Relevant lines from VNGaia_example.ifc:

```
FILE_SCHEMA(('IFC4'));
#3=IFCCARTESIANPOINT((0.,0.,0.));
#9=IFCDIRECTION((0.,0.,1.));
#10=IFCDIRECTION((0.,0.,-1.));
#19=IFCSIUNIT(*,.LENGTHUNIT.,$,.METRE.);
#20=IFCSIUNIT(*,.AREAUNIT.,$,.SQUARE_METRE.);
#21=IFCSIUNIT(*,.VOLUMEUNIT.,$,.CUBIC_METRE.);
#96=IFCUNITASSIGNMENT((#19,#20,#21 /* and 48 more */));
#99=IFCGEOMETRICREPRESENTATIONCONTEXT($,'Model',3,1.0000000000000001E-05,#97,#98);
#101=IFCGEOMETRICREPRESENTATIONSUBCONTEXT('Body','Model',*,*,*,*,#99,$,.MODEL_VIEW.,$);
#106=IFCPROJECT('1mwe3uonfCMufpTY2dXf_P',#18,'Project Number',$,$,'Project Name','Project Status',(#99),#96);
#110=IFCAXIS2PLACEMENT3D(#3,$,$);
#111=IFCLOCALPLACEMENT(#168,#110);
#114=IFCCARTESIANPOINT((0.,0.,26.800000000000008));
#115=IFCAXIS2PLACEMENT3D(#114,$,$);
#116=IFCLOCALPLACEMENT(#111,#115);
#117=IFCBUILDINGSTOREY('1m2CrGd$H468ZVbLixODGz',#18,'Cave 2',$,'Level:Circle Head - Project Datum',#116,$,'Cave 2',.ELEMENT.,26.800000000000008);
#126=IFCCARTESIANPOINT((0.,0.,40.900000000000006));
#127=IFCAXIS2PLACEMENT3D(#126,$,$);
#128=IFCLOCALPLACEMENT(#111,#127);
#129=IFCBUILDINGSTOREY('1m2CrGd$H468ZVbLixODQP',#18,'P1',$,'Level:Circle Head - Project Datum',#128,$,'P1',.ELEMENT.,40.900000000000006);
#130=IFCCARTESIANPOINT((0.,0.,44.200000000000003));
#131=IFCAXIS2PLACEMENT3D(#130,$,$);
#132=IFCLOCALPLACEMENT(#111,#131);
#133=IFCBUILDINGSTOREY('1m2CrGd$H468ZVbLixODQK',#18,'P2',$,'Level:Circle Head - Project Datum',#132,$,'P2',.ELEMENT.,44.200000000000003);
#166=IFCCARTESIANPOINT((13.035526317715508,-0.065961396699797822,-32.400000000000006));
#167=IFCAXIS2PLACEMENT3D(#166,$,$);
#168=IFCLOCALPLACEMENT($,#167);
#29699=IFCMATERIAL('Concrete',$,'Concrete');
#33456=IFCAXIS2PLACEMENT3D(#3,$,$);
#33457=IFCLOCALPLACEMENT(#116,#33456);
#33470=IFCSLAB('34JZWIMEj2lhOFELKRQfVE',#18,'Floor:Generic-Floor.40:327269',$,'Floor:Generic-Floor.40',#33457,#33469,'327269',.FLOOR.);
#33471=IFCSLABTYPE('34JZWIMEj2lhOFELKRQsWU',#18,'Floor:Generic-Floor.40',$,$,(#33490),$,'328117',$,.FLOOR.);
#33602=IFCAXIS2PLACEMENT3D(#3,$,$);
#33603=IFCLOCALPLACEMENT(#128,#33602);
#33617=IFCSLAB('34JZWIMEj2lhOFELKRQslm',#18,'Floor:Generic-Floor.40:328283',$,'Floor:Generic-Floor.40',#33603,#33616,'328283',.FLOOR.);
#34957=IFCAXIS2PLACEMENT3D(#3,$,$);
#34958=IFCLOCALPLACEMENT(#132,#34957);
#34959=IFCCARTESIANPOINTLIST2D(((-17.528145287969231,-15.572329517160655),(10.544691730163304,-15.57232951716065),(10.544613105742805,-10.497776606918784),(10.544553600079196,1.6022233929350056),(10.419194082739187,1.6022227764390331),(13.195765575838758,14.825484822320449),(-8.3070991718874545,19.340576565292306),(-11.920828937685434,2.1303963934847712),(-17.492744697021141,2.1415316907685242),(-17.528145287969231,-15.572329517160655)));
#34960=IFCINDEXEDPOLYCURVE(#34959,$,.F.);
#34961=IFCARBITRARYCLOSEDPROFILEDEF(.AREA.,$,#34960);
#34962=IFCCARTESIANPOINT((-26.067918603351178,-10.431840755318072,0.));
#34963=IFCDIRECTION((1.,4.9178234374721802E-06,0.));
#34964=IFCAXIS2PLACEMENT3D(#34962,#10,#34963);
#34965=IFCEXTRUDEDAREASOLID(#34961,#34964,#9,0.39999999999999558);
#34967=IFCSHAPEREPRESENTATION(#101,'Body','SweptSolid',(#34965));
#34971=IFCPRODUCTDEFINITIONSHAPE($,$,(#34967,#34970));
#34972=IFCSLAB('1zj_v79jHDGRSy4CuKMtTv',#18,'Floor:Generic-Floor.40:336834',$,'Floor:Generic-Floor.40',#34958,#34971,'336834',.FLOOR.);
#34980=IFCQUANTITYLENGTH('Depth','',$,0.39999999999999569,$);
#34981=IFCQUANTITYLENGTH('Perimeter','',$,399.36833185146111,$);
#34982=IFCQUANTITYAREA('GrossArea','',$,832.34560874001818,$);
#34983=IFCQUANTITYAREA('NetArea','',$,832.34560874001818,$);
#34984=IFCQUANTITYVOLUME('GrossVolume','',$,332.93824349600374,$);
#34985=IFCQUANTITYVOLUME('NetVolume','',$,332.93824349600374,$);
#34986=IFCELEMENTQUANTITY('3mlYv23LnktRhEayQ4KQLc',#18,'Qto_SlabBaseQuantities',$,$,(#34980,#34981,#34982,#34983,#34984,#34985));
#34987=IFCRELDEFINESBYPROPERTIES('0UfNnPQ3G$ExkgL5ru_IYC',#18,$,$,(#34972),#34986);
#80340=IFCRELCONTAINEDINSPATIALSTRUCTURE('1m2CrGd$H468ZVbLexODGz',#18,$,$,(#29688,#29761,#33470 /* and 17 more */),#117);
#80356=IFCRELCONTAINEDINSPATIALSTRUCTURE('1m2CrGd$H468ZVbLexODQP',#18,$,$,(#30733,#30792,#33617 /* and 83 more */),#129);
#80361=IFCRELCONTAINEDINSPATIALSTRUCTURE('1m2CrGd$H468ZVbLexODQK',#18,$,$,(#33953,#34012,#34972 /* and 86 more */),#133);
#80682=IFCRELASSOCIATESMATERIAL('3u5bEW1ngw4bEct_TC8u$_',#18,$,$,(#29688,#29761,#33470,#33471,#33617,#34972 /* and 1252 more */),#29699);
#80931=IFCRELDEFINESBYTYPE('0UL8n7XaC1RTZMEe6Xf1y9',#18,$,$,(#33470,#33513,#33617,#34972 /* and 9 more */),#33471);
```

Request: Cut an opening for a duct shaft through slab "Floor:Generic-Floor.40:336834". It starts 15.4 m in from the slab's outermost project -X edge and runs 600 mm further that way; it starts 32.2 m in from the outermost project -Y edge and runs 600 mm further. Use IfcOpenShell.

```python
import numpy as np
import ifcopenshell
import ifcopenshell.api.feature
import ifcopenshell.api.geometry
import ifcopenshell.api.pset
import ifcopenshell.api.root
import ifcopenshell.geom
import ifcopenshell.util.element
import ifcopenshell.util.placement
import ifcopenshell.util.representation
import ifcopenshell.util.shape
import ifcopenshell.util.unit

model = ifcopenshell.open("VNGaia_example.ifc")
unit_scale = ifcopenshell.util.unit.calculate_unit_scale(model)
area_scale = ifcopenshell.util.unit.calculate_unit_scale(model, "AREAUNIT")
volume_scale = ifcopenshell.util.unit.calculate_unit_scale(model, "VOLUMEUNIT")
settings = ifcopenshell.geom.settings()


def volume(element):
    """Net volume in cubic metres, openings subtracted."""
    shape = ifcopenshell.geom.create_shape(settings, element)
    return ifcopenshell.util.shape.get_volume(shape.geometry)


slab = model.by_id(34972)
before = volume(slab)

# Extent in the slab's own axes, in metres. The edges named are its -X and -Y sides.
slab_shape = ifcopenshell.geom.create_shape(settings, slab)
vertices = ifcopenshell.util.shape.get_vertices(slab_shape.geometry)
x_min, y_min, bottom = vertices.min(axis=0)
top = vertices[:, 2].max()

opening = ifcopenshell.api.root.create_entity(model, ifc_class="IfcOpeningElement", name="Duct shaft opening", predefined_type="OPENING")
context = ifcopenshell.util.representation.get_context(model, "Model", "Body", "MODEL_VIEW")
width, depth = 0.6, 0.6
outline = [(0.0, 0.0), (width, 0.0), (width, depth), (0.0, depth), (0.0, 0.0)]
# Overshoot both faces by 50 mm so the cut is clean.
shape = ifcopenshell.api.geometry.add_slab_representation(
    model, context=context, depth=top - bottom + 0.1, polyline=outline
)
ifcopenshell.api.geometry.assign_representation(model, product=opening, representation=shape)

matrix = ifcopenshell.util.placement.get_local_placement(slab.ObjectPlacement)
matrix[:, 3] = matrix @ np.append(np.array([x_min + 15.4, y_min + 32.2, bottom - 0.05]) / unit_scale, 1.0)
ifcopenshell.api.geometry.edit_object_placement(model, product=opening, matrix=matrix, is_si=False)
ifcopenshell.api.feature.add_feature(model, feature=opening, element=slab)

after = volume(slab)

# Update the slab's stored quantities.
qto = model.by_id(ifcopenshell.util.element.get_pset(slab, "Qto_SlabBaseQuantities", should_inherit=False)["id"])
ifcopenshell.api.pset.edit_qto(model, qto=qto, properties={
    "NetArea": after / (top - bottom) / area_scale,
    "NetVolume": after / volume_scale,
})

print(f"slab volume {before:.3f} -> {after:.3f} m3")

model.write("VNGaia_example_edited.ifc")
```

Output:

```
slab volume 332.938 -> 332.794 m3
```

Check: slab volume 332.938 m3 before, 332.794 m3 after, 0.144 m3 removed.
